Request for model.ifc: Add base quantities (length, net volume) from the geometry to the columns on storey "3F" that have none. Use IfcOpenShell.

First a look at what the model holds.

```python
import ifcopenshell
import ifcopenshell.util.element
import ifcopenshell.util.unit

model = ifcopenshell.open("model.ifc")
print(model.schema)
for unit_type in ("LENGTHUNIT", "AREAUNIT", "VOLUMEUNIT"):
    print(unit_type, ifcopenshell.util.unit.calculate_unit_scale(model, unit_type))
storey = next(s for s in model.by_type("IfcBuildingStorey") if s.Name == "3F")
columns = [e for e in ifcopenshell.util.element.get_decomposition(storey) if e.is_a("IfcColumn")]
for e in sorted(columns, key=lambda e: e.id()):
    print(e.id(), e.is_a(), e.Name, list(ifcopenshell.util.element.get_psets(e, qtos_only=True)), sep=" | ")
```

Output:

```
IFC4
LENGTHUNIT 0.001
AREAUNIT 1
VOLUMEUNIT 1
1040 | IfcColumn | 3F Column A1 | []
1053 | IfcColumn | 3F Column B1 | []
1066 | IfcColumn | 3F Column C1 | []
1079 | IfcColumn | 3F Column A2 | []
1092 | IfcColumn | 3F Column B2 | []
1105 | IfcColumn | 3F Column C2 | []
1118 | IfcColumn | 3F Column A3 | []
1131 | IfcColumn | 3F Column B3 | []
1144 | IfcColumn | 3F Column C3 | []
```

```python
import ifcopenshell
import ifcopenshell.api.pset
import ifcopenshell.geom
import ifcopenshell.util.element
import ifcopenshell.util.shape
import ifcopenshell.util.unit

model = ifcopenshell.open("model.ifc")
unit_scale = ifcopenshell.util.unit.calculate_unit_scale(model)
volume_scale = ifcopenshell.util.unit.calculate_unit_scale(model, "VOLUMEUNIT")
settings = ifcopenshell.geom.settings()

storey = next(s for s in model.by_type("IfcBuildingStorey") if s.Name == "3F")
columns = [e for e in ifcopenshell.util.element.get_decomposition(storey) if e.is_a("IfcColumn")]

for e in sorted(columns, key=lambda e: e.id()):
    if ifcopenshell.util.element.get_psets(e, qtos_only=True, should_inherit=False):
        continue
    # Geometry comes back in metres, in the element's own axes.
    shape = ifcopenshell.geom.create_shape(settings, e)
    values = {
        "Length": ifcopenshell.util.shape.get_z(shape.geometry) / unit_scale,
        "NetVolume": ifcopenshell.util.shape.get_volume(shape.geometry) / volume_scale,
    }
    qto = ifcopenshell.api.pset.add_qto(model, product=e, name="Qto_ColumnBaseQuantities")
    ifcopenshell.api.pset.edit_qto(model, qto=qto, properties=values)
    print(e.id(), {k: round(v, 3) for k, v in values.items()})

model.write("model_edited.ifc")
```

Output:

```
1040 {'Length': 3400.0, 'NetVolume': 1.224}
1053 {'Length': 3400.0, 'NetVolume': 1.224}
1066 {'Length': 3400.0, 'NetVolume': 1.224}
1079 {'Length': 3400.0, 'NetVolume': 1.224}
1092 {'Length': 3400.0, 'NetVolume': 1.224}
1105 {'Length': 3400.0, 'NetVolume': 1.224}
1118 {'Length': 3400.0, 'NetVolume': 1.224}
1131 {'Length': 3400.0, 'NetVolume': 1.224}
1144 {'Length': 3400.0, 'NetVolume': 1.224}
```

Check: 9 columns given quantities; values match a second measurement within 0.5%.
